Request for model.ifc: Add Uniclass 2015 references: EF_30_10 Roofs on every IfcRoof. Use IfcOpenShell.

First a look at what the model holds.

```python
import ifcopenshell

model = ifcopenshell.open("model.ifc")
print(model.schema)
print("classifications:", [c.Name for c in model.by_type("IfcClassification")])
for ifc_class in ("IfcDoor", "IfcRoof", "IfcStair", "IfcWall", "IfcWindow"):
    print(ifc_class, len(model.by_type(ifc_class)))
```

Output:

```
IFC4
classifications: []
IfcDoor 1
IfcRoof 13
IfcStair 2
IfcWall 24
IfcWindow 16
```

```python
import ifcopenshell
import ifcopenshell.api.classification

model = ifcopenshell.open("model.ifc")

system = ifcopenshell.api.classification.add_classification(model, classification="Uniclass 2015")

codes = {
    "IfcRoof": ("EF_30_10", "Roofs"),
}
for ifc_class, (code, name) in codes.items():
    products = model.by_type(ifc_class)
    ifcopenshell.api.classification.add_reference(
        model, products=products, classification=system, identification=code, name=name
    )
    print(code, len(products))

model.write("model_rev.ifc")
```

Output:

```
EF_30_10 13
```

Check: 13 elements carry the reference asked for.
